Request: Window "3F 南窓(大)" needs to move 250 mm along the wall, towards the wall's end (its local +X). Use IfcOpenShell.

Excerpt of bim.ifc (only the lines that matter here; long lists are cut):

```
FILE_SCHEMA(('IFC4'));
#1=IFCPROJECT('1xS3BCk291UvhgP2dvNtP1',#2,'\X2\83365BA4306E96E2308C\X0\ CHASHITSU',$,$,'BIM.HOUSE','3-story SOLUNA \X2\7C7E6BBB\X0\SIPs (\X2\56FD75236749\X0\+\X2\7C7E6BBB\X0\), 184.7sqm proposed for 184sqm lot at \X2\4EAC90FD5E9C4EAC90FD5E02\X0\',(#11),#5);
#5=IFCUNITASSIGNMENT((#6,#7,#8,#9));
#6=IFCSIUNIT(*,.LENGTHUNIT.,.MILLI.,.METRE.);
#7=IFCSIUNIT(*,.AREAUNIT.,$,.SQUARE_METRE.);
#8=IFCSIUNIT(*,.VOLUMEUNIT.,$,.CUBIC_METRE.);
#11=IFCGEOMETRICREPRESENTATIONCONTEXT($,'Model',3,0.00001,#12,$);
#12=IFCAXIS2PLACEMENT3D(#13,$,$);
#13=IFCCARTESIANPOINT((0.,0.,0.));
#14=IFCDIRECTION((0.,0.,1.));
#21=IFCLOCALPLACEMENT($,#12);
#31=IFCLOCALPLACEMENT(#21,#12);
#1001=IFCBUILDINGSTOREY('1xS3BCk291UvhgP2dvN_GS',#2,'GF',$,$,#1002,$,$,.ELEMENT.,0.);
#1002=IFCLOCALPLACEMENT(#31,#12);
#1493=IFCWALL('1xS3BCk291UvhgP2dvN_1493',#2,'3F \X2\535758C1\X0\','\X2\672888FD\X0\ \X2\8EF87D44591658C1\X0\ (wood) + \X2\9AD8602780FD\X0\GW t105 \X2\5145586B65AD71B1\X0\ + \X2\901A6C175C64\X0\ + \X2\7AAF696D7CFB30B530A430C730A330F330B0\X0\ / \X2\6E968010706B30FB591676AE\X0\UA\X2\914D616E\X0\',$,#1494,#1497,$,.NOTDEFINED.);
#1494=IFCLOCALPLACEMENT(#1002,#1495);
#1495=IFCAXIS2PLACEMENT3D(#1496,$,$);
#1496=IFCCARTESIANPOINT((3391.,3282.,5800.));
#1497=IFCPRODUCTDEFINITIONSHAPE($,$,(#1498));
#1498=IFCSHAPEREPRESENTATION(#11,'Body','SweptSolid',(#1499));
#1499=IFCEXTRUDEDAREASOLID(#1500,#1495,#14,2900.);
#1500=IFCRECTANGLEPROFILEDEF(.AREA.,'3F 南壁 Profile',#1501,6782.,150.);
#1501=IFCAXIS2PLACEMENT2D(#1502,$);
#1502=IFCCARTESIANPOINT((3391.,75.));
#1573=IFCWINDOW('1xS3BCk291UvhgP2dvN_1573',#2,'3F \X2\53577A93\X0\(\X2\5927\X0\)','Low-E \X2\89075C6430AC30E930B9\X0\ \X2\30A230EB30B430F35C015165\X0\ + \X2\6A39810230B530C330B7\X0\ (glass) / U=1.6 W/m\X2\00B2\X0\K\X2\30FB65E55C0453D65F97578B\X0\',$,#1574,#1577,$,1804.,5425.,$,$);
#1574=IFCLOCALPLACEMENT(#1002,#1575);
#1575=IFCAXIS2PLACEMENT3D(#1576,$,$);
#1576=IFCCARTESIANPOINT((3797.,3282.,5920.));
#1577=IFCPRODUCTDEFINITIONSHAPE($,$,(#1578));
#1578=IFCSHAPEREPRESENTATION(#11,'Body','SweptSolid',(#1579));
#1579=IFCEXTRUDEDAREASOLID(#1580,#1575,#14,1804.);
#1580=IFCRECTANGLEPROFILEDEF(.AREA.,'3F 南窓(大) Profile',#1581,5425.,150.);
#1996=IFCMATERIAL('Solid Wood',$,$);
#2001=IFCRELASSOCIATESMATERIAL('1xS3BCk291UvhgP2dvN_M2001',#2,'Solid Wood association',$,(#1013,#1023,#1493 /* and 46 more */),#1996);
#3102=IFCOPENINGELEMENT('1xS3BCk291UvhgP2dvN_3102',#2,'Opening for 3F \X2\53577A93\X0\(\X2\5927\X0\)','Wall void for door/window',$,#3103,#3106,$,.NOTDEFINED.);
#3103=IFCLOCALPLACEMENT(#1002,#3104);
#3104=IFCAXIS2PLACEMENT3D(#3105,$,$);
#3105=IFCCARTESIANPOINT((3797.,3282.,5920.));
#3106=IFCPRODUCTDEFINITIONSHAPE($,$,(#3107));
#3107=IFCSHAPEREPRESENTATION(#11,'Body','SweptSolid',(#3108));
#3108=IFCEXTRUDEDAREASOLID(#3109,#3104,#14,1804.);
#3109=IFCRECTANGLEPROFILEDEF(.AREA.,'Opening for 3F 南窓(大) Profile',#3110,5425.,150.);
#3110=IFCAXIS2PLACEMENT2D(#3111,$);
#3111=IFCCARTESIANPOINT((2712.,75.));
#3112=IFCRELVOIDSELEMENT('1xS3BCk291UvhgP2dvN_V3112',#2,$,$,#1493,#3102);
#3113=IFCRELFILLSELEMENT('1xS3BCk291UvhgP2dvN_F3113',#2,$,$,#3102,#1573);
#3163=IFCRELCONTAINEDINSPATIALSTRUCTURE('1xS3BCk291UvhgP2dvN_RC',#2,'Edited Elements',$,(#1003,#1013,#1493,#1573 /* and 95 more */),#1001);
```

```python
import ifcopenshell
import ifcopenshell.api.geometry
import ifcopenshell.util.placement

model = ifcopenshell.open("bim.ifc")

window = model.by_guid("1xS3BCk291UvhgP2dvN_1573")
opening = window.FillsVoids[0].RelatingOpeningElement
wall = opening.VoidsElements[0].RelatingBuildingElement

wall_matrix = ifcopenshell.util.placement.get_local_placement(wall.ObjectPlacement)
shift = wall_matrix[:3, 0] * 250.0
before = ifcopenshell.util.placement.get_local_placement(window.ObjectPlacement)[:3, 3].copy()

# The window is not placed relative to its opening, so move both.
for product in (opening, window):
    matrix = ifcopenshell.util.placement.get_local_placement(product.ObjectPlacement)
    matrix[:3, 3] += shift
    ifcopenshell.api.geometry.edit_object_placement(model, product=product, matrix=matrix, is_si=False)

after = ifcopenshell.util.placement.get_local_placement(window.ObjectPlacement)[:3, 3]
print("window moved by", (after - before).round(3) + 0.0)

model.write("bim_rev.ifc")
```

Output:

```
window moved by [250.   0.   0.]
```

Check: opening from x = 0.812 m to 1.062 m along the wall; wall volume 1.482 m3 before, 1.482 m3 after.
